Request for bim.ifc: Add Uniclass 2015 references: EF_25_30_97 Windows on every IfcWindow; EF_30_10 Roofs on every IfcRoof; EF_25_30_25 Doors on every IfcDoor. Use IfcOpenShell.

First a look at what the model holds.

```python
import ifcopenshell

model = ifcopenshell.open("bim.ifc")
print(model.schema)
print("classifications:", [c.Name for c in model.by_type("IfcClassification")])
for ifc_class in ("IfcDoor", "IfcRoof", "IfcStair", "IfcWall", "IfcWindow"):
    print(ifc_class, len(model.by_type(ifc_class)))
```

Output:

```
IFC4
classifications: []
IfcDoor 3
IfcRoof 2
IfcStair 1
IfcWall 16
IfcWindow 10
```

```python
import ifcopenshell
import ifcopenshell.api.classification

model = ifcopenshell.open("bim.ifc")

system = ifcopenshell.api.classification.add_classification(model, classification="Uniclass 2015")

codes = {
    "IfcWindow": ("EF_25_30_97", "Windows"),
    "IfcRoof": ("EF_30_10", "Roofs"),
    "IfcDoor": ("EF_25_30_25", "Doors"),
}
for ifc_class, (code, name) in codes.items():
    products = model.by_type(ifc_class)
    ifcopenshell.api.classification.add_reference(
        model, products=products, classification=system, identification=code, name=name
    )
    print(code, len(products))

model.write("bim_v2.ifc")
```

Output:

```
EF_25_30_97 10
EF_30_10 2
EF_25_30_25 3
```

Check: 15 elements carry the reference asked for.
